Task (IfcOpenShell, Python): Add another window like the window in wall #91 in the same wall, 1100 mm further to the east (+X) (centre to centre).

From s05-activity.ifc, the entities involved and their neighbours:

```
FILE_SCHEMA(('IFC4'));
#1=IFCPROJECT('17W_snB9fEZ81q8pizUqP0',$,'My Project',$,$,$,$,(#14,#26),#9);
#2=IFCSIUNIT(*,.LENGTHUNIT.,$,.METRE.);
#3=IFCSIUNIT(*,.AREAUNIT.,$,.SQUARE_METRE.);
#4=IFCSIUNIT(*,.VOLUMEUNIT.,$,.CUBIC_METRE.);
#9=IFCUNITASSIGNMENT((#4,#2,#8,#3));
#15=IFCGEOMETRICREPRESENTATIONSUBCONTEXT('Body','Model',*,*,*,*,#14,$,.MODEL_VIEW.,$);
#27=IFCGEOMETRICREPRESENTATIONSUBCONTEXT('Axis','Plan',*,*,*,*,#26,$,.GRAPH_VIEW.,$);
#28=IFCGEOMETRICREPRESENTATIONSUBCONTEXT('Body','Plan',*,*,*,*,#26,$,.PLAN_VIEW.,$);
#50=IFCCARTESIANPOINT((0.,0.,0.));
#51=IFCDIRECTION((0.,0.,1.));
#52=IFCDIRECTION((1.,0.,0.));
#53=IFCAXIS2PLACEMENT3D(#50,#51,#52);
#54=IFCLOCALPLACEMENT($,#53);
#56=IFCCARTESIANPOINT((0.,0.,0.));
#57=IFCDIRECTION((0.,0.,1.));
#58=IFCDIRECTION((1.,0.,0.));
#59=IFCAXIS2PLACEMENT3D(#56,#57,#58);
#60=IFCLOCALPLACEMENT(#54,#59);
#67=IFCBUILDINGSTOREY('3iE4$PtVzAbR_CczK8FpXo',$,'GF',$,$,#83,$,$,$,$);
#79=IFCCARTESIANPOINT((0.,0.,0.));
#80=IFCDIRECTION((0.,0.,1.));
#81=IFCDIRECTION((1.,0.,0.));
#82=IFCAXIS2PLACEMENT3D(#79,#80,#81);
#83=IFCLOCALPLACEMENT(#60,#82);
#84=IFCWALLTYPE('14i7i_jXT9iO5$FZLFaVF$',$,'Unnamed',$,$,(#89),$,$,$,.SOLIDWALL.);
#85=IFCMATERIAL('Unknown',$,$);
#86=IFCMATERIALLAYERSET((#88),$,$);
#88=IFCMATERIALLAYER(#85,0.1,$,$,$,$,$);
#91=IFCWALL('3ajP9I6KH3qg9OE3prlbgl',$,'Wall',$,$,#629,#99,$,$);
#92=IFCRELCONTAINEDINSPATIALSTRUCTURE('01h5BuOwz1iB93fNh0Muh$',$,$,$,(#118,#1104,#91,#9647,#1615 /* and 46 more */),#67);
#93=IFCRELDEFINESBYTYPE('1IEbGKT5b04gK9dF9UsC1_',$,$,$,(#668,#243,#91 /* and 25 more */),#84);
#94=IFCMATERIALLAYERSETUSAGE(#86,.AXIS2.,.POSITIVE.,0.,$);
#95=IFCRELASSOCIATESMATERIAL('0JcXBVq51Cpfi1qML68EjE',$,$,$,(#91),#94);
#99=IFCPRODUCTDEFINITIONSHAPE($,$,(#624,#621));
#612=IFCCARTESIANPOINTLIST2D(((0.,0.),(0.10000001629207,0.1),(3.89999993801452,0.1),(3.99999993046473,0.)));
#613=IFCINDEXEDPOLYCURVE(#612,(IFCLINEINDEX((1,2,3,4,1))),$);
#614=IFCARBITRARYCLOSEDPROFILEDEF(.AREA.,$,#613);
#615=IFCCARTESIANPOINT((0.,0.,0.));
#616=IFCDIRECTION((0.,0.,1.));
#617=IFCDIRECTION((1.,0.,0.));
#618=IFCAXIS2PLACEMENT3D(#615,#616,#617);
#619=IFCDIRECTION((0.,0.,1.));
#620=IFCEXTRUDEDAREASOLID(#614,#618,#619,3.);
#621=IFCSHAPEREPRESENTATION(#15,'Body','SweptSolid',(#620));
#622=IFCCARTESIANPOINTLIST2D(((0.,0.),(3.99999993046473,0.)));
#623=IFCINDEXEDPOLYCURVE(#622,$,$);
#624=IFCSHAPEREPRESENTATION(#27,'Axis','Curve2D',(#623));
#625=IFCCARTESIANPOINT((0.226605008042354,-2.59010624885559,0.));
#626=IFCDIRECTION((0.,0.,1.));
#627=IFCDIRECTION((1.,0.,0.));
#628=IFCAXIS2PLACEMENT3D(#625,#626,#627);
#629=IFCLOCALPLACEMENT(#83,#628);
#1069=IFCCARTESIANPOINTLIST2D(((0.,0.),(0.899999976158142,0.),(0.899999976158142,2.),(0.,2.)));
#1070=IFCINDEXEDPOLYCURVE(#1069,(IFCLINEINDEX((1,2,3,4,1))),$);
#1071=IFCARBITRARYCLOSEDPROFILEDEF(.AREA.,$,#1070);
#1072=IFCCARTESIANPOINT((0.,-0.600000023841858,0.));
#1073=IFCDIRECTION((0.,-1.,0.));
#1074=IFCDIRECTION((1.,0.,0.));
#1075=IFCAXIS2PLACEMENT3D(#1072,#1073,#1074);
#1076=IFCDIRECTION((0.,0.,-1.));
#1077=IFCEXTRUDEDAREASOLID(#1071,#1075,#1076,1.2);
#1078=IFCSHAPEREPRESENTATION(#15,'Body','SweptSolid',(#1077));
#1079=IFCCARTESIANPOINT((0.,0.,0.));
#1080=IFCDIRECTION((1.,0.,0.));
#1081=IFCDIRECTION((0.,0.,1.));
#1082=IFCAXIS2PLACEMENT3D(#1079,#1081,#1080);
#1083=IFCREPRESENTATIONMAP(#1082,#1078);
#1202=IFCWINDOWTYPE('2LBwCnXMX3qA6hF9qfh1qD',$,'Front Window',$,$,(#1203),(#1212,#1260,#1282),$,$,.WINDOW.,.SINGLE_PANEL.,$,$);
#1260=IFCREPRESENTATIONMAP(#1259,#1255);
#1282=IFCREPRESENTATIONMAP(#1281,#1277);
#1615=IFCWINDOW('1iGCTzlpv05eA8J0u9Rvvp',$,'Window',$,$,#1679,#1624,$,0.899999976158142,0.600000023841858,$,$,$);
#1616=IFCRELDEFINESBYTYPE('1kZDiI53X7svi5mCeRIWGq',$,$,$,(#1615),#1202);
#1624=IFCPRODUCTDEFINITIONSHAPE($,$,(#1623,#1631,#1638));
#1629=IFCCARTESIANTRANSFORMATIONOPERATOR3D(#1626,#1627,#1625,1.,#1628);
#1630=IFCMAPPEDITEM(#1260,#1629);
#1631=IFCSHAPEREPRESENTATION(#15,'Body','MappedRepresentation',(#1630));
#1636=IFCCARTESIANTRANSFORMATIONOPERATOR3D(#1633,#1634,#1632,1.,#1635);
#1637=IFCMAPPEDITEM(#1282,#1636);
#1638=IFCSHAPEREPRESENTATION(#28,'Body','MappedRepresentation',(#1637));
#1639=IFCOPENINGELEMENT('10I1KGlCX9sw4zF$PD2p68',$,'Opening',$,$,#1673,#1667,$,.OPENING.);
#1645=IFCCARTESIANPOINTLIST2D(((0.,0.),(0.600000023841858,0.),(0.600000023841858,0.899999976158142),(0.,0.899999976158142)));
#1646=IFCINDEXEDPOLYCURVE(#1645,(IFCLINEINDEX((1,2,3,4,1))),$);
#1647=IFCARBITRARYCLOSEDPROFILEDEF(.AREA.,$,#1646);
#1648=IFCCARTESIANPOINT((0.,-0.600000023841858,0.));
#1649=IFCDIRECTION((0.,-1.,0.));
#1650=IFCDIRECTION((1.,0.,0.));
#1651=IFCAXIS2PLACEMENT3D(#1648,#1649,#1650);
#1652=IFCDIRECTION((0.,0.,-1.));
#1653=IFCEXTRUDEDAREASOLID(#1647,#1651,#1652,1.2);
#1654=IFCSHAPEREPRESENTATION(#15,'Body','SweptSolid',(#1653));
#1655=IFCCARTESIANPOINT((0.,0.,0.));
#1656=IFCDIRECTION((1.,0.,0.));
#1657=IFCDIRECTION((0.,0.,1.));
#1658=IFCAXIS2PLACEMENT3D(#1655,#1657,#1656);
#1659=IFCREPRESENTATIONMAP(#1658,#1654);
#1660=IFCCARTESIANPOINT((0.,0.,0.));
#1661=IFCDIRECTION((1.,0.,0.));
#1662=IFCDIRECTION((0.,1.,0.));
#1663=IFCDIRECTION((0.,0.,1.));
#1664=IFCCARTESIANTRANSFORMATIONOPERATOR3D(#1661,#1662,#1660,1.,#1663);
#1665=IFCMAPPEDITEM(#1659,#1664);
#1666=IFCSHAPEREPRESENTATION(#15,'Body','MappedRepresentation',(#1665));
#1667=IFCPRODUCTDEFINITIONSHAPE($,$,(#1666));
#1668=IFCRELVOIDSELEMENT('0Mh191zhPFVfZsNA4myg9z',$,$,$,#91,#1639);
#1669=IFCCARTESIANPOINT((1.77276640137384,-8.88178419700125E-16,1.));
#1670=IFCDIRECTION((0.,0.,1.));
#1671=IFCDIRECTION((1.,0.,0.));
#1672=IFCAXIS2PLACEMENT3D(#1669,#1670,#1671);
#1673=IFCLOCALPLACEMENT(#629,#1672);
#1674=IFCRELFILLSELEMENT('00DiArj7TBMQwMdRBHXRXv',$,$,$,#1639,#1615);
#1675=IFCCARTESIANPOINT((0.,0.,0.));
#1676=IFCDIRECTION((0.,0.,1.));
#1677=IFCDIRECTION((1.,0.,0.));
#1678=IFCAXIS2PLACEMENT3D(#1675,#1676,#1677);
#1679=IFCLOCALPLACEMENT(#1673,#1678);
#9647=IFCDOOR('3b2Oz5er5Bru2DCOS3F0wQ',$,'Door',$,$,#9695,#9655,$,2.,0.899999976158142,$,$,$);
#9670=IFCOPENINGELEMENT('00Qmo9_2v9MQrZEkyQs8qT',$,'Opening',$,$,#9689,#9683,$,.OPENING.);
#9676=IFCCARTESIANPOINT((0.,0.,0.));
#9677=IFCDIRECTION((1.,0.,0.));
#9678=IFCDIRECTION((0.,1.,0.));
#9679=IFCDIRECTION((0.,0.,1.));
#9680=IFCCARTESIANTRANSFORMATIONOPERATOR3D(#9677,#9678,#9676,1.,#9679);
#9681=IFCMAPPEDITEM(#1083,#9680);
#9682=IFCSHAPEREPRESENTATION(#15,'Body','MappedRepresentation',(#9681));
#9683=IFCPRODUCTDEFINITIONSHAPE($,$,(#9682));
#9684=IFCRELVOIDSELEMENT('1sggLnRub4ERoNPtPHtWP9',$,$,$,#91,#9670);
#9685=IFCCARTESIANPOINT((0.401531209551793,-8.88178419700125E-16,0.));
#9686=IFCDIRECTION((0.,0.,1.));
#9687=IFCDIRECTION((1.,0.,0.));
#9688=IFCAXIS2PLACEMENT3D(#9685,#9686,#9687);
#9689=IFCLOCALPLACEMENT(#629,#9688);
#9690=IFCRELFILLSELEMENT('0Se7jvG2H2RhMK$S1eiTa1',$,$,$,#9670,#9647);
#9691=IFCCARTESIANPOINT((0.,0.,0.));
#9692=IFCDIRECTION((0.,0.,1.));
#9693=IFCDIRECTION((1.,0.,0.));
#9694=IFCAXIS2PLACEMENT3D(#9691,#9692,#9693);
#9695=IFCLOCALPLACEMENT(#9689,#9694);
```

```python
import ifcopenshell
import ifcopenshell.api.feature
import ifcopenshell.api.geometry
import ifcopenshell.api.root
import ifcopenshell.geom
import ifcopenshell.util.element
import ifcopenshell.util.placement
import ifcopenshell.util.shape
import ifcopenshell.util.unit

model = ifcopenshell.open("s05-activity.ifc")
unit_scale = ifcopenshell.util.unit.calculate_unit_scale(model)
settings = ifcopenshell.geom.settings()


def volume(element):
    """Net volume in cubic metres, openings subtracted."""
    shape = ifcopenshell.geom.create_shape(settings, element)
    return ifcopenshell.util.shape.get_volume(shape.geometry)


window = model.by_id(1615)
opening = window.FillsVoids[0].RelatingOpeningElement
wall = opening.VoidsElements[0].RelatingBuildingElement
before = volume(wall)
shift = ifcopenshell.util.placement.get_local_placement(wall.ObjectPlacement)[:3, 0] * 1.1 / unit_scale

# copy_class copies the void relationship, type, container and properties, but no geometry.
new_opening = ifcopenshell.api.root.copy_class(model, product=opening)
new_opening.Representation = ifcopenshell.util.element.copy_deep(
    model, opening.Representation, exclude=["IfcGeometricRepresentationContext", "IfcRepresentationMap"]
)
new_window = ifcopenshell.api.root.copy_class(model, product=window)
new_window.Representation = ifcopenshell.util.element.copy_deep(
    model, window.Representation, exclude=["IfcGeometricRepresentationContext", "IfcRepresentationMap"]
)
ifcopenshell.api.feature.add_filling(model, opening=new_opening, element=new_window)

for old, new in ((opening, new_opening), (window, new_window)):
    matrix = ifcopenshell.util.placement.get_local_placement(old.ObjectPlacement)
    matrix[:3, 3] += shift
    ifcopenshell.api.geometry.edit_object_placement(model, product=new, matrix=matrix, is_si=False)

after = volume(wall)

print(f"wall volume {before:.3f} -> {after:.3f} m3")

model.write("s05-activity_edited.ifc")
```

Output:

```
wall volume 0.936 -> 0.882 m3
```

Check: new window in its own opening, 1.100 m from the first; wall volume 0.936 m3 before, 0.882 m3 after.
